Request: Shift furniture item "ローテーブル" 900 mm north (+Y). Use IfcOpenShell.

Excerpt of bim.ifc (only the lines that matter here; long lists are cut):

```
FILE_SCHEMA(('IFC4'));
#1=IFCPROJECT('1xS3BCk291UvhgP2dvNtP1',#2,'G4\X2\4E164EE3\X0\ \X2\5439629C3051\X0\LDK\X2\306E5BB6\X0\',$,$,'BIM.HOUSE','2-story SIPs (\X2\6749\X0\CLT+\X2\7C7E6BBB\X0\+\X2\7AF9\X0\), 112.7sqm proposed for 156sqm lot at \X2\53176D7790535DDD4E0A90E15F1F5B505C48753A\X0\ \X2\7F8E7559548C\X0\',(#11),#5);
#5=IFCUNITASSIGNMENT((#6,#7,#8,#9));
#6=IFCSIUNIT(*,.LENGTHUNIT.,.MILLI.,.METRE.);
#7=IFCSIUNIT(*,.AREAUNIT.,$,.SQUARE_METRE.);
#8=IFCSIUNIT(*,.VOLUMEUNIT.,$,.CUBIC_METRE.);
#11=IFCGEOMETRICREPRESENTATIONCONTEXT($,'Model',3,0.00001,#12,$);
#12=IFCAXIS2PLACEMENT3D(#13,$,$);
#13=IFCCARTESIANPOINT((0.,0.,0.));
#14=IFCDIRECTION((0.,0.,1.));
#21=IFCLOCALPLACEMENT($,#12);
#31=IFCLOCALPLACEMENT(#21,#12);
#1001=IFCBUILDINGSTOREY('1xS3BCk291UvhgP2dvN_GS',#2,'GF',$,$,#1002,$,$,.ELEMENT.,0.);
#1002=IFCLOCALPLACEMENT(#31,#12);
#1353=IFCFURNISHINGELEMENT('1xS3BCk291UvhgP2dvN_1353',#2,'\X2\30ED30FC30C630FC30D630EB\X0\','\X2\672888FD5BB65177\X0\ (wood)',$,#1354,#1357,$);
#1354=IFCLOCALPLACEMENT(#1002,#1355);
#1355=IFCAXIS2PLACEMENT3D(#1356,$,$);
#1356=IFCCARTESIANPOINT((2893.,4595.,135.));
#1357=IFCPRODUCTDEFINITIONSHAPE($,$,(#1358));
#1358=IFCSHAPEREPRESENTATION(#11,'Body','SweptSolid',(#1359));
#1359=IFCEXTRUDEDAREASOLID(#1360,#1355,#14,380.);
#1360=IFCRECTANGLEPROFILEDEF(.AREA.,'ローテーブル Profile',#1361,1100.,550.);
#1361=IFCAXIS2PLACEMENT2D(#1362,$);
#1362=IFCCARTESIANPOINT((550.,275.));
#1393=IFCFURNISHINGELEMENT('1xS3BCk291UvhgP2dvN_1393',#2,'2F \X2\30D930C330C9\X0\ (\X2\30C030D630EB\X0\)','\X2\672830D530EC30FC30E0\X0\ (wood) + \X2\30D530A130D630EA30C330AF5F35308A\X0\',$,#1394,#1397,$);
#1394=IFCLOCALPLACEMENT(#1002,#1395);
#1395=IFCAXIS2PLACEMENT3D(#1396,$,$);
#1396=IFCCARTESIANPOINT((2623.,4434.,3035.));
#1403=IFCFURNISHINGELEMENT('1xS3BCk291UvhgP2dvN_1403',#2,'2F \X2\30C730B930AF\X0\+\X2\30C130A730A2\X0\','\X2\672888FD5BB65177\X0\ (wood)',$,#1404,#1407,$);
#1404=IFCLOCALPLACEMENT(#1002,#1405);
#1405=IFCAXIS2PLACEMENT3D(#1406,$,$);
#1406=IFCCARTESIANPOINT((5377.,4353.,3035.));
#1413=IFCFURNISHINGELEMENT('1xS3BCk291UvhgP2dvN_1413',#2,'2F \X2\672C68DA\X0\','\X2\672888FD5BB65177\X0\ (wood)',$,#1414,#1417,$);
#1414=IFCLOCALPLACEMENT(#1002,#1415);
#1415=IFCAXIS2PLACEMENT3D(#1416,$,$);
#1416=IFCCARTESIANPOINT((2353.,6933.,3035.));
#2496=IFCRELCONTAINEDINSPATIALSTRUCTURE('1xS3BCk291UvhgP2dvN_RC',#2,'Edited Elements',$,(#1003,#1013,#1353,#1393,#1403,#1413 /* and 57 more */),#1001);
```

```python
import ifcopenshell
import ifcopenshell.api.geometry
import ifcopenshell.util.placement

model = ifcopenshell.open("bim.ifc")

item = model.by_guid("1xS3BCk291UvhgP2dvN_1353")
matrix = ifcopenshell.util.placement.get_local_placement(item.ObjectPlacement)
matrix[1, 3] += 900.0
ifcopenshell.api.geometry.edit_object_placement(model, product=item, matrix=matrix, is_si=False)

print(ifcopenshell.util.placement.get_local_placement(item.ObjectPlacement).round(3) + 0.0)

model.write("bim_v2.ifc")
```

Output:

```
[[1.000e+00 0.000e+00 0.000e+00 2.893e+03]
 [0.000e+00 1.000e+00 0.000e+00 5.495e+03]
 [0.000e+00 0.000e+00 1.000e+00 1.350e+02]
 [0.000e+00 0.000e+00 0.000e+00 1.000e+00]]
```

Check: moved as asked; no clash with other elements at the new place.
